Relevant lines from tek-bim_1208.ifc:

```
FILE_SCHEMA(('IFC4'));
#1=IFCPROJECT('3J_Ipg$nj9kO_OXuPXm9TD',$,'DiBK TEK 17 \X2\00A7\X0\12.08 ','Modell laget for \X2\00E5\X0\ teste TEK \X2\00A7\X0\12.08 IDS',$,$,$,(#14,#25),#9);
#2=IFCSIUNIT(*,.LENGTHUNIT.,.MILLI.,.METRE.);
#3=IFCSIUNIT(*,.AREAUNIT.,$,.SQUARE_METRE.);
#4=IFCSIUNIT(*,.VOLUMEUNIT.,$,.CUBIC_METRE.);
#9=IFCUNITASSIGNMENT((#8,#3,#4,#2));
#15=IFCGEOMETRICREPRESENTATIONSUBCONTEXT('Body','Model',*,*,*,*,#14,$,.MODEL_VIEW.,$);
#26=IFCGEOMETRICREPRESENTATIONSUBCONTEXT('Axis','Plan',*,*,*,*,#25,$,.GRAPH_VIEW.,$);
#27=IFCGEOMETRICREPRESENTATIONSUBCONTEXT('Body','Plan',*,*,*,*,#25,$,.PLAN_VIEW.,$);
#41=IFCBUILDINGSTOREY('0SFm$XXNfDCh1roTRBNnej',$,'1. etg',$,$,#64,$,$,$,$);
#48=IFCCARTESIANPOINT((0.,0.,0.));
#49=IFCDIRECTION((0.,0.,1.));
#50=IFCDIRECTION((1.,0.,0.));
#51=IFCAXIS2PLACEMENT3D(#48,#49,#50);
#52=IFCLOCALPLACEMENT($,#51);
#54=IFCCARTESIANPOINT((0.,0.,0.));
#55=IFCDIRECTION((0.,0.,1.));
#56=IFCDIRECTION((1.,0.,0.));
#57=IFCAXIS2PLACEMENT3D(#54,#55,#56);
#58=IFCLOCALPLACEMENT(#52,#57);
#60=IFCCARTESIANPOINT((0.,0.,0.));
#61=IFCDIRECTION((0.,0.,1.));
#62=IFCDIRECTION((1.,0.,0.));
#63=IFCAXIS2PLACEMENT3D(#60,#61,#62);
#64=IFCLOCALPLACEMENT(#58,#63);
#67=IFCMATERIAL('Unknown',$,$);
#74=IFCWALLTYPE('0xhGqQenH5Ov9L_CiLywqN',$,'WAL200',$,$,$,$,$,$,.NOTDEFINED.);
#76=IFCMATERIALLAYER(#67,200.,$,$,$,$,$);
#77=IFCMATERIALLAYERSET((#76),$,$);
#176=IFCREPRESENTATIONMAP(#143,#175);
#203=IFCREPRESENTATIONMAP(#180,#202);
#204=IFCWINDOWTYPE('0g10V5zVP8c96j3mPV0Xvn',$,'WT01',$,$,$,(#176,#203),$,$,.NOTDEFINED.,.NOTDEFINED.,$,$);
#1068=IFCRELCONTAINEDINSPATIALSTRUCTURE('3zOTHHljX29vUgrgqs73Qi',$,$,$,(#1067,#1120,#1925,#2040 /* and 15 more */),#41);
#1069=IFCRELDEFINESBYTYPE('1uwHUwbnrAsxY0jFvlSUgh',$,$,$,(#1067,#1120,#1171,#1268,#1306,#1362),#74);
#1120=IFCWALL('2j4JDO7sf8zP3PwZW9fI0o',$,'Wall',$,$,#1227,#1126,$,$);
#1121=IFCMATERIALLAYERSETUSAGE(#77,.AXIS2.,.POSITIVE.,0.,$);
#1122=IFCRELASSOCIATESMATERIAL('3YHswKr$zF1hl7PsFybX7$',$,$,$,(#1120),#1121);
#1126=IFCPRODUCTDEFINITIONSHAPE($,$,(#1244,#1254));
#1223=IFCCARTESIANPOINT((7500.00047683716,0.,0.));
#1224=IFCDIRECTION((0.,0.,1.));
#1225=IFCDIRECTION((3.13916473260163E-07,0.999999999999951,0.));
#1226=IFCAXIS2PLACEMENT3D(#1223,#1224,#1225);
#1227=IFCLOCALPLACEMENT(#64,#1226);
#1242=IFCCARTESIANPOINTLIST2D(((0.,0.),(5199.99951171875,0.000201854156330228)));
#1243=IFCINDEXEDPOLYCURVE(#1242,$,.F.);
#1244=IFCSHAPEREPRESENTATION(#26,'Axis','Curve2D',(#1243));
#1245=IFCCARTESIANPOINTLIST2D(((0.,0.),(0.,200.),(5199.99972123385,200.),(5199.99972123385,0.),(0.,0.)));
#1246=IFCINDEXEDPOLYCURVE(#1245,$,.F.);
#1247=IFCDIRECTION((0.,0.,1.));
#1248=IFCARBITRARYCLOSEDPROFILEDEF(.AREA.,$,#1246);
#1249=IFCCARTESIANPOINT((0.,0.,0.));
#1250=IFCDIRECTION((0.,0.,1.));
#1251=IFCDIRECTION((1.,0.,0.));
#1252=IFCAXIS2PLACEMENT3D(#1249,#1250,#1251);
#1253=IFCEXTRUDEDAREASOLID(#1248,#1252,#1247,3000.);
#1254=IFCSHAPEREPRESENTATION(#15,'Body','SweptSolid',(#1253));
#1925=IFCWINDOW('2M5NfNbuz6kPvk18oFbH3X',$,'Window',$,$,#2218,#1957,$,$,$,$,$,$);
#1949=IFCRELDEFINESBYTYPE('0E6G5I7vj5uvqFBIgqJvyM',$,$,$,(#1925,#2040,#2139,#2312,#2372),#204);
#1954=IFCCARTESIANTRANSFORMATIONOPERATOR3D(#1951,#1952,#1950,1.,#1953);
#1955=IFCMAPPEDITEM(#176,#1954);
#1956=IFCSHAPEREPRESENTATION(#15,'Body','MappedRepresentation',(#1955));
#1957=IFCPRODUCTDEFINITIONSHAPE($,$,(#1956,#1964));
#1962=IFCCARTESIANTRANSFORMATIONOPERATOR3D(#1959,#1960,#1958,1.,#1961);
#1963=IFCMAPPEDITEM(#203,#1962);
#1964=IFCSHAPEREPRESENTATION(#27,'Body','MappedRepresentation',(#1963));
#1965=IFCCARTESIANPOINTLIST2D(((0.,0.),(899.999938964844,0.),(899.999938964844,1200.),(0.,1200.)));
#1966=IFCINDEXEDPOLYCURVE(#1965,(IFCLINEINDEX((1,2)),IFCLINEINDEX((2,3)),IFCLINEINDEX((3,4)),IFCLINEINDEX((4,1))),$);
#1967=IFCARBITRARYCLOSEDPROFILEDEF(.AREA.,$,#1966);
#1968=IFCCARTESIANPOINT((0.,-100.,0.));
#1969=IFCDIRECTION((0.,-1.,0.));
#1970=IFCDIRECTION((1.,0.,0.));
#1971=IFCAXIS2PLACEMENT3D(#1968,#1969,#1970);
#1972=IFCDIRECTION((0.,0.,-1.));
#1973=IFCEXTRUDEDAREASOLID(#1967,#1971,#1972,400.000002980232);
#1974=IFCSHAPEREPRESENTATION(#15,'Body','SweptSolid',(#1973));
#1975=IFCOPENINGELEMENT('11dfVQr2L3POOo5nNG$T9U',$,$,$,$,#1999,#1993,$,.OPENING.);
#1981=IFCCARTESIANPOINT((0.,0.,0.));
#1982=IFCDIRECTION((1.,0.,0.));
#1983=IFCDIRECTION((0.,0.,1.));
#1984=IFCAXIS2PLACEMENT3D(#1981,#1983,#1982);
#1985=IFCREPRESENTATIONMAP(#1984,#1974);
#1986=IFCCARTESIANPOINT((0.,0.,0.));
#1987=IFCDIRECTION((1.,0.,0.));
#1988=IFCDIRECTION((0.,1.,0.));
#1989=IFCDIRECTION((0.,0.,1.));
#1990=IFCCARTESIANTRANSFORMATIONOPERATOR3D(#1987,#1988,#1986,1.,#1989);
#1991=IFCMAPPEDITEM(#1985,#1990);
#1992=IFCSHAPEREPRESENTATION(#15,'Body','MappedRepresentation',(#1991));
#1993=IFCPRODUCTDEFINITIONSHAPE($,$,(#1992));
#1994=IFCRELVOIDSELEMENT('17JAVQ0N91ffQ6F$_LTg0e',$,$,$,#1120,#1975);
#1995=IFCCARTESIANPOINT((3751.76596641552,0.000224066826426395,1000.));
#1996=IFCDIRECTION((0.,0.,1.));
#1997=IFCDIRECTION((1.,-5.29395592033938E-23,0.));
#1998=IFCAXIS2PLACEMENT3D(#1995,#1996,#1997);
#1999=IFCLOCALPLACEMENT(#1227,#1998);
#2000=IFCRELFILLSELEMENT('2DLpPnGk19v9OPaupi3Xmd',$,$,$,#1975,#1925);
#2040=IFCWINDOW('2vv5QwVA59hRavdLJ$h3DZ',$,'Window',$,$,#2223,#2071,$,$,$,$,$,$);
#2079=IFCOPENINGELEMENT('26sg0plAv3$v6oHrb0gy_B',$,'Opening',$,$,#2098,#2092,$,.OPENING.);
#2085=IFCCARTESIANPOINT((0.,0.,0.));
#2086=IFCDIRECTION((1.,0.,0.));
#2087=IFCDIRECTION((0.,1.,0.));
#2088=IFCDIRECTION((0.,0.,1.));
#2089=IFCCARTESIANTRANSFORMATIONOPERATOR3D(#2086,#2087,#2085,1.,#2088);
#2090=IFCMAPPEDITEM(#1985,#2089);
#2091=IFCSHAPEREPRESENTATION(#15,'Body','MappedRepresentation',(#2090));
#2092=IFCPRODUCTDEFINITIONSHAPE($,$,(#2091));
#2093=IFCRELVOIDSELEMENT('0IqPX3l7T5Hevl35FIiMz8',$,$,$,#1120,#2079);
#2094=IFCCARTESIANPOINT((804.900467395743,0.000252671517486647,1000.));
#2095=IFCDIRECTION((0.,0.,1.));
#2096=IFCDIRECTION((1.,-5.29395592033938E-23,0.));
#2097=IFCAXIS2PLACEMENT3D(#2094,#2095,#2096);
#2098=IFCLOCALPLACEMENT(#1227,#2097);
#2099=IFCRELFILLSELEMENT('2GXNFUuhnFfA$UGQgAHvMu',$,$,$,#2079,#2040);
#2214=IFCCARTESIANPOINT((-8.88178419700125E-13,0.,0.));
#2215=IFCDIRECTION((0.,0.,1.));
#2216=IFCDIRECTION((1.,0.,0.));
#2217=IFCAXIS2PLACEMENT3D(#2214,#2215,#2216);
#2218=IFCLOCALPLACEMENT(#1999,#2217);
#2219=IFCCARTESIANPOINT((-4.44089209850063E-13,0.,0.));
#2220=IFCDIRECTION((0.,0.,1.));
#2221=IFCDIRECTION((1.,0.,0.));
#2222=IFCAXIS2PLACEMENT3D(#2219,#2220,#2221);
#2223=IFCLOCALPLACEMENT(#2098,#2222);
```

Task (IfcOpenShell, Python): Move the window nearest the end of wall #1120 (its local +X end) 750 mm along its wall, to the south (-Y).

```python
import ifcopenshell
import ifcopenshell.api.geometry
import ifcopenshell.util.placement
import ifcopenshell.util.unit

model = ifcopenshell.open("tek-bim_1208.ifc")
unit_scale = ifcopenshell.util.unit.calculate_unit_scale(model)

window = model.by_guid("2M5NfNbuz6kPvk18oFbH3X")
opening = window.FillsVoids[0].RelatingOpeningElement
wall = opening.VoidsElements[0].RelatingBuildingElement

wall_matrix = ifcopenshell.util.placement.get_local_placement(wall.ObjectPlacement)
shift = wall_matrix[:3, 0] * -0.75 / unit_scale
before = ifcopenshell.util.placement.get_local_placement(window.ObjectPlacement)[:3, 3].copy()

# The window is placed relative to its opening, so it follows when the opening moves.
matrix = ifcopenshell.util.placement.get_local_placement(opening.ObjectPlacement)
matrix[:3, 3] += shift
ifcopenshell.api.geometry.edit_object_placement(
    model, product=opening, matrix=matrix, is_si=False, should_transform_children=True
)

after = ifcopenshell.util.placement.get_local_placement(window.ObjectPlacement)[:3, 3]
print("window moved by", (after - before).round(3) + 0.0)

model.write("tek-bim_1208_rev.ifc")
```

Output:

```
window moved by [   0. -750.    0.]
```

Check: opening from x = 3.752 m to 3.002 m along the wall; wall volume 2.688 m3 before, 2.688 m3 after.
